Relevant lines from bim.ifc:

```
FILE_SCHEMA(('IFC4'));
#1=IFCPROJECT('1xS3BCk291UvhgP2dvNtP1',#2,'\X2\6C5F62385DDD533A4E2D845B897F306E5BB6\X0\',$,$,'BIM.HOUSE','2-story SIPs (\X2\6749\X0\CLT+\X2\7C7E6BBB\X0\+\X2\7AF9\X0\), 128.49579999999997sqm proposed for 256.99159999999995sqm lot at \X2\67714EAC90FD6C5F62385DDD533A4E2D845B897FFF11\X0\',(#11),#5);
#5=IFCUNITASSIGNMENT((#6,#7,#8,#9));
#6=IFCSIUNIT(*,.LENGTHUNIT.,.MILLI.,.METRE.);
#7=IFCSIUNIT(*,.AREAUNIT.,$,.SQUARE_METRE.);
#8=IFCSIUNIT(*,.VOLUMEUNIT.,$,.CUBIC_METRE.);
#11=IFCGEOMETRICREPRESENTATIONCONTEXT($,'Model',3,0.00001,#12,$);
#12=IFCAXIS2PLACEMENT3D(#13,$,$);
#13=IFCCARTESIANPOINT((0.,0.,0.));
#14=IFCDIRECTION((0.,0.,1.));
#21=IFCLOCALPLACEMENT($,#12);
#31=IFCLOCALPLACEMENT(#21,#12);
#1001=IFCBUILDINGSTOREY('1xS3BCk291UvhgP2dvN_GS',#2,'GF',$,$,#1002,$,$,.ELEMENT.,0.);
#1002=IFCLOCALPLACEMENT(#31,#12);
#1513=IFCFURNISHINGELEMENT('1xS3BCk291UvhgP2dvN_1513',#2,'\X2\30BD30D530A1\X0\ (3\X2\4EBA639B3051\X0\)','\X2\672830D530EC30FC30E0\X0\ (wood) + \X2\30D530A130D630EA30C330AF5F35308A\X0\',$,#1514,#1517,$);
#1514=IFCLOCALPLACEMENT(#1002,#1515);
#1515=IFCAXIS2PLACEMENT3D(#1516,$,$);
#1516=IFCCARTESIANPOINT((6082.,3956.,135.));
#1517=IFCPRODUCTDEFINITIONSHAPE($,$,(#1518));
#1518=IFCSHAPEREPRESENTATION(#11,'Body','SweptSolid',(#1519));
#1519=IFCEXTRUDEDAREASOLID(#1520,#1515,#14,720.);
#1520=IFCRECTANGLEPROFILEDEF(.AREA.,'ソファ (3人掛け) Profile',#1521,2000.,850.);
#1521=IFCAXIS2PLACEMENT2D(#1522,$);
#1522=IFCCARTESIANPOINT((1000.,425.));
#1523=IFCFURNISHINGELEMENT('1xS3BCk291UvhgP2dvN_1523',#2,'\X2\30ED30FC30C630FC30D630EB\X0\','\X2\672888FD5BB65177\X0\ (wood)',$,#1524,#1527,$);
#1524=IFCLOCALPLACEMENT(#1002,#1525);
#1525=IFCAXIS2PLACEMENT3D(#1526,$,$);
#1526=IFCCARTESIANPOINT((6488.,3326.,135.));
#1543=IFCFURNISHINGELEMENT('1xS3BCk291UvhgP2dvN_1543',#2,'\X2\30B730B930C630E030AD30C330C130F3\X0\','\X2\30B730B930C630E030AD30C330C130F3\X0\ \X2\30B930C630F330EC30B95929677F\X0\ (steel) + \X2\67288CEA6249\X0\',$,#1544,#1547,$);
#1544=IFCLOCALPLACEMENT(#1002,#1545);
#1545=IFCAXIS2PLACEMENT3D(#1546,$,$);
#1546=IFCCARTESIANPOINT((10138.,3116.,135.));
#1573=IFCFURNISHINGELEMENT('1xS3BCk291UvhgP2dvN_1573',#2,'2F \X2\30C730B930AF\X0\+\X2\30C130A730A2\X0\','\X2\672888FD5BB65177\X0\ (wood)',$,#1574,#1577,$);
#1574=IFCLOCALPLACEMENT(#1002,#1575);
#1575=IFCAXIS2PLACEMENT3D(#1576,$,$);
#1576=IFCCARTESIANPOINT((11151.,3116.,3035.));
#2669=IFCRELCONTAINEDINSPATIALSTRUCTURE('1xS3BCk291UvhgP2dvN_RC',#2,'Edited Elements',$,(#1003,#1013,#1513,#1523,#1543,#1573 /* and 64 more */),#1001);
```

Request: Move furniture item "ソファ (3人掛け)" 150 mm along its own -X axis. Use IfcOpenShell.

```python
import ifcopenshell
import ifcopenshell.api.geometry
import ifcopenshell.util.placement
import ifcopenshell.util.unit

model = ifcopenshell.open("bim.ifc")
unit_scale = ifcopenshell.util.unit.calculate_unit_scale(model)

item = model.by_guid("1xS3BCk291UvhgP2dvN_1513")
matrix = ifcopenshell.util.placement.get_local_placement(item.ObjectPlacement)
matrix[:3, 3] -= matrix[:3, 0] * 0.15 / unit_scale
ifcopenshell.api.geometry.edit_object_placement(model, product=item, matrix=matrix, is_si=False)

print(ifcopenshell.util.placement.get_local_placement(item.ObjectPlacement).round(3) + 0.0)

model.write("bim_rev.ifc")
```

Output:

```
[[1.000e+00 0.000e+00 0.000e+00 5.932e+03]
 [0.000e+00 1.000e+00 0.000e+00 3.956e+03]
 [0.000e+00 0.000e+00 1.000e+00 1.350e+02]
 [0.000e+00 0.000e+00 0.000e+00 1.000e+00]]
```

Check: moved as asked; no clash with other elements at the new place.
